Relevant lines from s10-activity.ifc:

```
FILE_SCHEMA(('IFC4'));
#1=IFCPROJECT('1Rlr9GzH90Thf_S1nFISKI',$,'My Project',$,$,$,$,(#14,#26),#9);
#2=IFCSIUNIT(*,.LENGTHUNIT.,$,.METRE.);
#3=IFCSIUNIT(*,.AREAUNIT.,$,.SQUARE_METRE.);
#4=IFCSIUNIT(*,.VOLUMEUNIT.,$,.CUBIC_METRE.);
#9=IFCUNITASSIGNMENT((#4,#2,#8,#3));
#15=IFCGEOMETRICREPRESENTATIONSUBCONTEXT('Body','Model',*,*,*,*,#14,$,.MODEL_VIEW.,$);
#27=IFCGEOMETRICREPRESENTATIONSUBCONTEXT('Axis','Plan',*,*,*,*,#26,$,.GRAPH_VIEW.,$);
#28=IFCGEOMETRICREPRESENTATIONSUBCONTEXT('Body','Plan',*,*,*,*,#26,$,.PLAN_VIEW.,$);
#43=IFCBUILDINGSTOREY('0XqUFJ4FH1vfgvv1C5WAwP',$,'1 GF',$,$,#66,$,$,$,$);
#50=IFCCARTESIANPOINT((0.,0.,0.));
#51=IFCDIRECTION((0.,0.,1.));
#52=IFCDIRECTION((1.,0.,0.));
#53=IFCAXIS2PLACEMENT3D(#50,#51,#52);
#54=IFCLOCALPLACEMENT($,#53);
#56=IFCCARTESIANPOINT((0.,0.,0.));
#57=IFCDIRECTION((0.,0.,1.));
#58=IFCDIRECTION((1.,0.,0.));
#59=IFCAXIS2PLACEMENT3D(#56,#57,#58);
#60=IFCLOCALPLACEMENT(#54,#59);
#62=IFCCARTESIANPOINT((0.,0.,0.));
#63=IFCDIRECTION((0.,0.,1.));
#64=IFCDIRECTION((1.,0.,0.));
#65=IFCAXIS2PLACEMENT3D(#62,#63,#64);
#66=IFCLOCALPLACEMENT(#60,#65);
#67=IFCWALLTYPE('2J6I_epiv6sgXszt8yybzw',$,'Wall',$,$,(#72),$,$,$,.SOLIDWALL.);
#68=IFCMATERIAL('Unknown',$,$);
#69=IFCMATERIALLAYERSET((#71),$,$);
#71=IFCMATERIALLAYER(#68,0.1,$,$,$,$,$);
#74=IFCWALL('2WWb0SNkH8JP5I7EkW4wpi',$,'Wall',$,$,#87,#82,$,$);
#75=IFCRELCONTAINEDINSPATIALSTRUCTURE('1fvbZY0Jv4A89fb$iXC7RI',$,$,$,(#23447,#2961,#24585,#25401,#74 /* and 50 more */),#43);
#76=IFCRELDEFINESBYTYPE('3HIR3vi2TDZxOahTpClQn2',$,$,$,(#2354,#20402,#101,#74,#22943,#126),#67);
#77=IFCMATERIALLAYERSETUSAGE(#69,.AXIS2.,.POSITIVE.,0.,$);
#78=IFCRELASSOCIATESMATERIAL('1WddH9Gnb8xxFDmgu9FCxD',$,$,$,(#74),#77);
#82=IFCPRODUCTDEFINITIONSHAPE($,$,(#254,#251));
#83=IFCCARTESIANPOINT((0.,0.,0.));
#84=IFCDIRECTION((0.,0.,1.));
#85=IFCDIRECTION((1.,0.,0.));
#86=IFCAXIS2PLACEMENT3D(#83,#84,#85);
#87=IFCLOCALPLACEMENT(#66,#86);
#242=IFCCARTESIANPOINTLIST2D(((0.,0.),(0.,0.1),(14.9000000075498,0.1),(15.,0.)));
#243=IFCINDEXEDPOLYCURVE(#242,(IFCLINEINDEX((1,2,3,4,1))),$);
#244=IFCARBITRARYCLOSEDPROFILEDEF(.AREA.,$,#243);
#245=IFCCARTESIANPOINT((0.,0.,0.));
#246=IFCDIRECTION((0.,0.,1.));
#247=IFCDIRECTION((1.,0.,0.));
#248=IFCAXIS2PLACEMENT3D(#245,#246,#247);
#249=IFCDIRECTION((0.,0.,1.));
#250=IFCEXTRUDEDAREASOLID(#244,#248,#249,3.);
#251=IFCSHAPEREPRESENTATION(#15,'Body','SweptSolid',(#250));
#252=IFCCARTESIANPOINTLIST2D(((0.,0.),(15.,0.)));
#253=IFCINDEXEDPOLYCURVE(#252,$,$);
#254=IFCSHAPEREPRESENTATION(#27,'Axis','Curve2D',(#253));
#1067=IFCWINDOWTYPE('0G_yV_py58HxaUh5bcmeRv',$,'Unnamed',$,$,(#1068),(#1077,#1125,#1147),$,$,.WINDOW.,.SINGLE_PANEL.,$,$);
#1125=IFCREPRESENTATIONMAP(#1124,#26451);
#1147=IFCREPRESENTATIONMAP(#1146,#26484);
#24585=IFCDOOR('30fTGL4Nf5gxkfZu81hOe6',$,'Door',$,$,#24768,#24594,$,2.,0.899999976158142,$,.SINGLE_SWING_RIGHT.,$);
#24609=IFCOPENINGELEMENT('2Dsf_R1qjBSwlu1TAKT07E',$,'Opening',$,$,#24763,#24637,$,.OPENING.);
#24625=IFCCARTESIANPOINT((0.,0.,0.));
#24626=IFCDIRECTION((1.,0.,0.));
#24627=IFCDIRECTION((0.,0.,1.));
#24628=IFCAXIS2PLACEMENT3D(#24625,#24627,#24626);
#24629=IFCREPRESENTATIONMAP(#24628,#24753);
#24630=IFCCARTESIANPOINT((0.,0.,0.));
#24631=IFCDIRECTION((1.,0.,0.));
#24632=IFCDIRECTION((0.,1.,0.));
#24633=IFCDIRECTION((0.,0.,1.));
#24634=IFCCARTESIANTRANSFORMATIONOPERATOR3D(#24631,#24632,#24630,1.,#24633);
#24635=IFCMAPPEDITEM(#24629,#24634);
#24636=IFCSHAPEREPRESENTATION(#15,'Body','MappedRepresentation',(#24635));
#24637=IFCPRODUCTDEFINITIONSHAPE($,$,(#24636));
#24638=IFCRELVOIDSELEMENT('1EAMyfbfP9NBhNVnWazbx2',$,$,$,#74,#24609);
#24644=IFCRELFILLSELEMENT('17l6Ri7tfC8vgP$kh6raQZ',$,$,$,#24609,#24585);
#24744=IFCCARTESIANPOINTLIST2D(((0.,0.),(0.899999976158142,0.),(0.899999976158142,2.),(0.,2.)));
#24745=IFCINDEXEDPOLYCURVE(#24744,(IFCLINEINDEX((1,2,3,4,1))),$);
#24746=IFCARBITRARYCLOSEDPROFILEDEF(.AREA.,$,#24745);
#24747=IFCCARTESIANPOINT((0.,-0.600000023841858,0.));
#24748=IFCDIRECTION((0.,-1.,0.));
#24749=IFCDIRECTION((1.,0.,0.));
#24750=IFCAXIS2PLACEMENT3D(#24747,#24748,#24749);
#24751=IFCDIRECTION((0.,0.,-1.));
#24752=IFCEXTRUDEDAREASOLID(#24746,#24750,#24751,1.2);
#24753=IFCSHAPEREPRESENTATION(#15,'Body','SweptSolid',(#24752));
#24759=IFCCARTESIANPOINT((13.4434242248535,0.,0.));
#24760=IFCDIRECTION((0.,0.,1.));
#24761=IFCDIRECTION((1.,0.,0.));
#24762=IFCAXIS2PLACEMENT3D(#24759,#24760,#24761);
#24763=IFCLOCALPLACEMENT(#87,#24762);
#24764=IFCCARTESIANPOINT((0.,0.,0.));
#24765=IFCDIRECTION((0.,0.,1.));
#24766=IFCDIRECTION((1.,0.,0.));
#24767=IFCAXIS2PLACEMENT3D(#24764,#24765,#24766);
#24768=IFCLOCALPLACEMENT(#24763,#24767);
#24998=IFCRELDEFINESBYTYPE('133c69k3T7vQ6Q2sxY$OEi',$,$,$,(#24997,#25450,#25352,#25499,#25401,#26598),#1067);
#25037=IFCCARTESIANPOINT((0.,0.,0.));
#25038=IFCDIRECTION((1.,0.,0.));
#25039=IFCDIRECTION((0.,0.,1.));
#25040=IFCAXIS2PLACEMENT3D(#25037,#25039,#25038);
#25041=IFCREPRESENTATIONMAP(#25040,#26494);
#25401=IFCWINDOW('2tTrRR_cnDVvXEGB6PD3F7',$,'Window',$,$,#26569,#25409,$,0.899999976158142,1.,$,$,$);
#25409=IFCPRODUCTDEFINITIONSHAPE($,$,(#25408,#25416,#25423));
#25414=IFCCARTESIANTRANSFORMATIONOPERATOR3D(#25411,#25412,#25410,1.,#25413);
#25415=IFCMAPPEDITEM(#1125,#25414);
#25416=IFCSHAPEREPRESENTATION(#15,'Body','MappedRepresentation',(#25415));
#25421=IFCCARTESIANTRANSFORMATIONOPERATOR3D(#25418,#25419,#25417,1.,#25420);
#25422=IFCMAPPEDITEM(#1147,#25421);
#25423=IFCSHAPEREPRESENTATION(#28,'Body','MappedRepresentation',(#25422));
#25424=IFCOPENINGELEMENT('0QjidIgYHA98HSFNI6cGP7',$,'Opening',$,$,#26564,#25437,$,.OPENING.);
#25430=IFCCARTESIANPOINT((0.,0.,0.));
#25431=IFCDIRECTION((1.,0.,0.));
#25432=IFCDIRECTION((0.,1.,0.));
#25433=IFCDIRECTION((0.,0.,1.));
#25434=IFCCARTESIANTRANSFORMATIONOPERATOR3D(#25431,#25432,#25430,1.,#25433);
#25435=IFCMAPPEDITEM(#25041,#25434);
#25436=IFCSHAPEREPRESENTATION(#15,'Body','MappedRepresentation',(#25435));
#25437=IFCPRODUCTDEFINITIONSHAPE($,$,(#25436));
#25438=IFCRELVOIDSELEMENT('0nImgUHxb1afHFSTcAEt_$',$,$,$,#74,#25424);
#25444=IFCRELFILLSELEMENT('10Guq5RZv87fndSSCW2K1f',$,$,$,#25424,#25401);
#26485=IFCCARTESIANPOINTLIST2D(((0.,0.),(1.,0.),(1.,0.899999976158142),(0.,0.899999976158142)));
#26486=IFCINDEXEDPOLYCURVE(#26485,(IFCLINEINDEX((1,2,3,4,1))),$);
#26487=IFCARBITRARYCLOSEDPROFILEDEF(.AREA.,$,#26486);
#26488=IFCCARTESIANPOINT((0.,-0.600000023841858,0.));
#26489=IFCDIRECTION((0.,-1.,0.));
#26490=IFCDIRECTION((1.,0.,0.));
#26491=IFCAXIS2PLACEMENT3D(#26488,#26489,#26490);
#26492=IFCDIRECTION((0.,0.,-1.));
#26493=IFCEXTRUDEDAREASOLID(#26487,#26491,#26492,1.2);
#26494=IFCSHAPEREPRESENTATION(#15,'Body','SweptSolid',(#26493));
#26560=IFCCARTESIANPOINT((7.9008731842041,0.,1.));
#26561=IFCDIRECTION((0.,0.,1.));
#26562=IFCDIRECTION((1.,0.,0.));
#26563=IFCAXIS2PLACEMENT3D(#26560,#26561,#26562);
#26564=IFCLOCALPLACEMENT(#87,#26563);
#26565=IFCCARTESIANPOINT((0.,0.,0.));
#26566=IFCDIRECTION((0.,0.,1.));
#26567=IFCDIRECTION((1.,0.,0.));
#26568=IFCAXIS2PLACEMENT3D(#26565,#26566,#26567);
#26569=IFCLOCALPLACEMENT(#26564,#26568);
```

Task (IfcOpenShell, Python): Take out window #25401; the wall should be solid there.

```python
import ifcopenshell
import ifcopenshell.api.feature
import ifcopenshell.api.root
import ifcopenshell.geom
import ifcopenshell.util.shape

model = ifcopenshell.open("s10-activity.ifc")
settings = ifcopenshell.geom.settings()


def volume(element):
    """Net volume in cubic metres, openings subtracted."""
    shape = ifcopenshell.geom.create_shape(settings, element)
    return ifcopenshell.util.shape.get_volume(shape.geometry)


window = model.by_guid("2tTrRR_cnDVvXEGB6PD3F7")
opening = window.FillsVoids[0].RelatingOpeningElement
wall = opening.VoidsElements[0].RelatingBuildingElement
before = volume(wall)

ifcopenshell.api.root.remove_product(model, product=window)
ifcopenshell.api.feature.remove_feature(model, feature=opening)

after = volume(wall)

print(f"wall volume {before:.3f} -> {after:.3f} m3")

model.write("s10-activity_edited.ifc")
```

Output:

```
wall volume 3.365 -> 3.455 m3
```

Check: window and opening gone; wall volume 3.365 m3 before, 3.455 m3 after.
